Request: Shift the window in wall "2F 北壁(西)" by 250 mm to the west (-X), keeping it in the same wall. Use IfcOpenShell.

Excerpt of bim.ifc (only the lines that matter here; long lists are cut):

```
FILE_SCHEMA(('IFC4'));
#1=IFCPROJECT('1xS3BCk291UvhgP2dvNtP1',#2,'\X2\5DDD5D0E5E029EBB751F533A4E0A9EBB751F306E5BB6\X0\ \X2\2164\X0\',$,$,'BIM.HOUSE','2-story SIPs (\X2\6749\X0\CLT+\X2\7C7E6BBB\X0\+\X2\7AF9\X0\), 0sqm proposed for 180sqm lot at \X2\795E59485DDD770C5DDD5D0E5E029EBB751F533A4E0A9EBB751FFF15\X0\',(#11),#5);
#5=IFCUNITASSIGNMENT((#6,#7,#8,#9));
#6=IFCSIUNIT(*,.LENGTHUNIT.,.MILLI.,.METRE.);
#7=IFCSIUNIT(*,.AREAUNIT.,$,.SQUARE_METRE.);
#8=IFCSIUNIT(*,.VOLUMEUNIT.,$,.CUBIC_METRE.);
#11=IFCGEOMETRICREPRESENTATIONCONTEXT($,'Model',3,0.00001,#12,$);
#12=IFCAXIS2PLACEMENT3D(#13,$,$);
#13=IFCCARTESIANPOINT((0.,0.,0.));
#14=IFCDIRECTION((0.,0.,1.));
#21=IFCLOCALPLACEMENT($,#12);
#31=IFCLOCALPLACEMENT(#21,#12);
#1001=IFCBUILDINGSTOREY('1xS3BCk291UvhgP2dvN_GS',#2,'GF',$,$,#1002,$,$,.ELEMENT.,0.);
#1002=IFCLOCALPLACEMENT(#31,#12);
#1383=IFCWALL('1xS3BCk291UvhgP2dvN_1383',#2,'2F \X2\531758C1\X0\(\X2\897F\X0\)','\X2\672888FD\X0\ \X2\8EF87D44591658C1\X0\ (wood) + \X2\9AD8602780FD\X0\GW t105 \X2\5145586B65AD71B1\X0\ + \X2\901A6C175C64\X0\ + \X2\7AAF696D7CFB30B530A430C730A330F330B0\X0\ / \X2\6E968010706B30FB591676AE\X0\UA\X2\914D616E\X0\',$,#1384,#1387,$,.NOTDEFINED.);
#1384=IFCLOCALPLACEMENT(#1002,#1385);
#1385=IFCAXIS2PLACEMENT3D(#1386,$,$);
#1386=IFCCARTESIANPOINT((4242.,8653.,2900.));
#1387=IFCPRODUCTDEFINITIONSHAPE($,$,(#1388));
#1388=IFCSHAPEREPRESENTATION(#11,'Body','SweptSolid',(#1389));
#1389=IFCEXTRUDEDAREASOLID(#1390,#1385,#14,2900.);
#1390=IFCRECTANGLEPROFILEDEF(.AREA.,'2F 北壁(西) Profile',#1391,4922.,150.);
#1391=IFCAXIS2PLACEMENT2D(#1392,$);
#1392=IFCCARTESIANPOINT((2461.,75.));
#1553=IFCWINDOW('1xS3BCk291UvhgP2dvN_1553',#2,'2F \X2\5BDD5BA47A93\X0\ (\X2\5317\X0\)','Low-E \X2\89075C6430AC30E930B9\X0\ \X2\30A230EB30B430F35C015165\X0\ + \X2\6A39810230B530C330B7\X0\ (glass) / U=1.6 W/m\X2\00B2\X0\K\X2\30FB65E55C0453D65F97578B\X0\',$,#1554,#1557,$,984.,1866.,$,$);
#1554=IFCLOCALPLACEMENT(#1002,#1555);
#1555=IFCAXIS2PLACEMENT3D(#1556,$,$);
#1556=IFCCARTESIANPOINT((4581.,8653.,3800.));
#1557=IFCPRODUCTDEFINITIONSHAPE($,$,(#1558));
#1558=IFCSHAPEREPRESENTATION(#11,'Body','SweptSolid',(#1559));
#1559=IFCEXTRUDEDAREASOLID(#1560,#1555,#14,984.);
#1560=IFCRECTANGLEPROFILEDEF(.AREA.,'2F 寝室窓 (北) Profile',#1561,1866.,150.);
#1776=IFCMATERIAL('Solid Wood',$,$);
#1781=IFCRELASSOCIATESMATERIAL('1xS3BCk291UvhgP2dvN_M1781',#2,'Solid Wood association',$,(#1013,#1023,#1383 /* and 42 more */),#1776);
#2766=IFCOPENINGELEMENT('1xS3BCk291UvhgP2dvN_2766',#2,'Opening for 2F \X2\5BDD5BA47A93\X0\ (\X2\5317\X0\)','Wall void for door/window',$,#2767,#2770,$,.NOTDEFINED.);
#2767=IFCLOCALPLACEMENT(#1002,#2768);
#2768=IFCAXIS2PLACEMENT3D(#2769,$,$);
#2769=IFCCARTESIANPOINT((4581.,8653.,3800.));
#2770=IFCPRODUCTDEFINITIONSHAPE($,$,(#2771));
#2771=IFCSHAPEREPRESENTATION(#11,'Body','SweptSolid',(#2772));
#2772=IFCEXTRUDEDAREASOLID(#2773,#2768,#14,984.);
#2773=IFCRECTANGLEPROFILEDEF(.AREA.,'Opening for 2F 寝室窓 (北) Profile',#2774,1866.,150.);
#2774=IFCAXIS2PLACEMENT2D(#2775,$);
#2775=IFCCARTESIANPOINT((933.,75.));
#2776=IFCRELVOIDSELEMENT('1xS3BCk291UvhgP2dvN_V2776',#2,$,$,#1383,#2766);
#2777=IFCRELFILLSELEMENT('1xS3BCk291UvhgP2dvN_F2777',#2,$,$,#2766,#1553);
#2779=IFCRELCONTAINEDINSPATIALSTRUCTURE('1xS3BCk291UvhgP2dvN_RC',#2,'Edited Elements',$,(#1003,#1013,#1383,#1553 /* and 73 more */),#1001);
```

```python
import ifcopenshell
import ifcopenshell.api.geometry
import ifcopenshell.util.placement
import ifcopenshell.util.unit

model = ifcopenshell.open("bim.ifc")
unit_scale = ifcopenshell.util.unit.calculate_unit_scale(model)

window = model.by_guid("1xS3BCk291UvhgP2dvN_1553")
opening = window.FillsVoids[0].RelatingOpeningElement
wall = opening.VoidsElements[0].RelatingBuildingElement

wall_matrix = ifcopenshell.util.placement.get_local_placement(wall.ObjectPlacement)
shift = wall_matrix[:3, 0] * -0.25 / unit_scale
before = ifcopenshell.util.placement.get_local_placement(window.ObjectPlacement)[:3, 3].copy()

# The window is not placed relative to its opening, so move both.
for product in (opening, window):
    matrix = ifcopenshell.util.placement.get_local_placement(product.ObjectPlacement)
    matrix[:3, 3] += shift
    ifcopenshell.api.geometry.edit_object_placement(model, product=product, matrix=matrix, is_si=False)

after = ifcopenshell.util.placement.get_local_placement(window.ObjectPlacement)[:3, 3]
print("window moved by", (after - before).round(3) + 0.0)

model.write("bim_edited.ifc")
```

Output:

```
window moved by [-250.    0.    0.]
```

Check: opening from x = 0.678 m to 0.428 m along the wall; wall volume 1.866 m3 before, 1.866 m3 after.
